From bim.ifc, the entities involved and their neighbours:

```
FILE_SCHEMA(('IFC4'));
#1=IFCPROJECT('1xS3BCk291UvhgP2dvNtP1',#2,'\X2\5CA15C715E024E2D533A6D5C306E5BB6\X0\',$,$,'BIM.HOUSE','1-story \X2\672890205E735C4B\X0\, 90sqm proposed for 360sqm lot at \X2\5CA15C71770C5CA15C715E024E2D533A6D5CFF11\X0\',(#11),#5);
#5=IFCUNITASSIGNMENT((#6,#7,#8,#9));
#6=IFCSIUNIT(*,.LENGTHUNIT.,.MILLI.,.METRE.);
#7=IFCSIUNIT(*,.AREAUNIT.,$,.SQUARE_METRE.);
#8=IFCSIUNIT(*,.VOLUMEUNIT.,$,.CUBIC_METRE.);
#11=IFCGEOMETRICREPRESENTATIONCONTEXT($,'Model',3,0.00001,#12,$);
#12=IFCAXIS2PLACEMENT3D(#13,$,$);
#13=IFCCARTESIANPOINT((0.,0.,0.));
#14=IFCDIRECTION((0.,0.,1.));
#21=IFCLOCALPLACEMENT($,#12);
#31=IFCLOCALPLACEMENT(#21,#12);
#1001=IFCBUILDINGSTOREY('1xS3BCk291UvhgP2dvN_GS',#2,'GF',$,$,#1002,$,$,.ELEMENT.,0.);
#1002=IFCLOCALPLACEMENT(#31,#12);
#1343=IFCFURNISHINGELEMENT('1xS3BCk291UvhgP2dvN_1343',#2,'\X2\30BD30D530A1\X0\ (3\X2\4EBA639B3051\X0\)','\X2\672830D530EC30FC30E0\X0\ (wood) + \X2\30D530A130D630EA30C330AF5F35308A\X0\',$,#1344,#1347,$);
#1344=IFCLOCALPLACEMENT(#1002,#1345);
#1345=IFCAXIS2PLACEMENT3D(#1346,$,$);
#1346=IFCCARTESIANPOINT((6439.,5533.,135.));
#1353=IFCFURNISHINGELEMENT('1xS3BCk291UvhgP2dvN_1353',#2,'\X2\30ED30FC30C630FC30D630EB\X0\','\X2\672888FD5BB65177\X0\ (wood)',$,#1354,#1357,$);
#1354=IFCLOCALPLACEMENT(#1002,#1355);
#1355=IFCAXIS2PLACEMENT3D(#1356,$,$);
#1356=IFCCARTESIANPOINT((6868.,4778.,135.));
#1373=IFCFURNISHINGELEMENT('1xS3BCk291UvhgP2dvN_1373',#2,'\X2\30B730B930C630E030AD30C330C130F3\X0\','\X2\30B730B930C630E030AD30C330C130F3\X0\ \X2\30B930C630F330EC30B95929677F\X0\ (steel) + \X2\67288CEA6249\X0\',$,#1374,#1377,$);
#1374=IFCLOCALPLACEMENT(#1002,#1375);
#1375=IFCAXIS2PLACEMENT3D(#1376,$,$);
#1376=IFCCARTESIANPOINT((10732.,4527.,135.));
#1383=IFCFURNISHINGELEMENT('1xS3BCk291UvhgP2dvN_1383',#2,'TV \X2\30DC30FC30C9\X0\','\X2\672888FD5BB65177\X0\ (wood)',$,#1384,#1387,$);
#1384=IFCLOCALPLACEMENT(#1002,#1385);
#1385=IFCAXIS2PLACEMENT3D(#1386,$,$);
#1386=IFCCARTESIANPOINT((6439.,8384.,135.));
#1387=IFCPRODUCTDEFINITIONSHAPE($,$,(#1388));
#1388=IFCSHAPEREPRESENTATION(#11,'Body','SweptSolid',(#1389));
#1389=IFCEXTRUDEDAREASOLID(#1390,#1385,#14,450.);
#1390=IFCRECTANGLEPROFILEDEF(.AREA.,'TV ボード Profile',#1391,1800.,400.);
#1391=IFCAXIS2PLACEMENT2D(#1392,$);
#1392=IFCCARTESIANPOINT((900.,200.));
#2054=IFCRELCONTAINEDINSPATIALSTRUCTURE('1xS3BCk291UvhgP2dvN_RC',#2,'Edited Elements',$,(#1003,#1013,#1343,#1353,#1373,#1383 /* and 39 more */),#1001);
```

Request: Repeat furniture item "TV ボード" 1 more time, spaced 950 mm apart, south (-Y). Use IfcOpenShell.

```python
import numpy as np
import ifcopenshell
import ifcopenshell.api.geometry
import ifcopenshell.api.root
import ifcopenshell.util.element
import ifcopenshell.util.placement

model = ifcopenshell.open("bim.ifc")


def reuse_history(source, copy):
    """copy_class also copies each property set's owner history, people and application; keep the originals."""
    for rel in copy.IsDefinedBy:
        if rel.is_a("IfcRelDefinesByProperties") and (history := rel.RelatingPropertyDefinition.OwnerHistory):
            rel.RelatingPropertyDefinition.OwnerHistory = source.OwnerHistory
            ifcopenshell.util.element.remove_deep2(model, history)


source = model.by_guid("1xS3BCk291UvhgP2dvN_1383")
base = ifcopenshell.util.placement.get_local_placement(source.ObjectPlacement)
step = np.array([0.0, -1.0, 0.0]) * 950.0

for i in range(1, 2):
    copy = ifcopenshell.api.root.copy_class(model, product=source)
    copy.Representation = ifcopenshell.util.element.copy_deep(
        model, source.Representation, exclude=["IfcGeometricRepresentationContext", "IfcRepresentationMap"]
    )
    reuse_history(source, copy)
    matrix = base.copy()
    matrix[:3, 3] += i * step
    print("added at", matrix[:3, 3].round(3) + 0.0)
    ifcopenshell.api.geometry.edit_object_placement(model, product=copy, matrix=matrix, is_si=False)

model.write("bim-out.ifc")
```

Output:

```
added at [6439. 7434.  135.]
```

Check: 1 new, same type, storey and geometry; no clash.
